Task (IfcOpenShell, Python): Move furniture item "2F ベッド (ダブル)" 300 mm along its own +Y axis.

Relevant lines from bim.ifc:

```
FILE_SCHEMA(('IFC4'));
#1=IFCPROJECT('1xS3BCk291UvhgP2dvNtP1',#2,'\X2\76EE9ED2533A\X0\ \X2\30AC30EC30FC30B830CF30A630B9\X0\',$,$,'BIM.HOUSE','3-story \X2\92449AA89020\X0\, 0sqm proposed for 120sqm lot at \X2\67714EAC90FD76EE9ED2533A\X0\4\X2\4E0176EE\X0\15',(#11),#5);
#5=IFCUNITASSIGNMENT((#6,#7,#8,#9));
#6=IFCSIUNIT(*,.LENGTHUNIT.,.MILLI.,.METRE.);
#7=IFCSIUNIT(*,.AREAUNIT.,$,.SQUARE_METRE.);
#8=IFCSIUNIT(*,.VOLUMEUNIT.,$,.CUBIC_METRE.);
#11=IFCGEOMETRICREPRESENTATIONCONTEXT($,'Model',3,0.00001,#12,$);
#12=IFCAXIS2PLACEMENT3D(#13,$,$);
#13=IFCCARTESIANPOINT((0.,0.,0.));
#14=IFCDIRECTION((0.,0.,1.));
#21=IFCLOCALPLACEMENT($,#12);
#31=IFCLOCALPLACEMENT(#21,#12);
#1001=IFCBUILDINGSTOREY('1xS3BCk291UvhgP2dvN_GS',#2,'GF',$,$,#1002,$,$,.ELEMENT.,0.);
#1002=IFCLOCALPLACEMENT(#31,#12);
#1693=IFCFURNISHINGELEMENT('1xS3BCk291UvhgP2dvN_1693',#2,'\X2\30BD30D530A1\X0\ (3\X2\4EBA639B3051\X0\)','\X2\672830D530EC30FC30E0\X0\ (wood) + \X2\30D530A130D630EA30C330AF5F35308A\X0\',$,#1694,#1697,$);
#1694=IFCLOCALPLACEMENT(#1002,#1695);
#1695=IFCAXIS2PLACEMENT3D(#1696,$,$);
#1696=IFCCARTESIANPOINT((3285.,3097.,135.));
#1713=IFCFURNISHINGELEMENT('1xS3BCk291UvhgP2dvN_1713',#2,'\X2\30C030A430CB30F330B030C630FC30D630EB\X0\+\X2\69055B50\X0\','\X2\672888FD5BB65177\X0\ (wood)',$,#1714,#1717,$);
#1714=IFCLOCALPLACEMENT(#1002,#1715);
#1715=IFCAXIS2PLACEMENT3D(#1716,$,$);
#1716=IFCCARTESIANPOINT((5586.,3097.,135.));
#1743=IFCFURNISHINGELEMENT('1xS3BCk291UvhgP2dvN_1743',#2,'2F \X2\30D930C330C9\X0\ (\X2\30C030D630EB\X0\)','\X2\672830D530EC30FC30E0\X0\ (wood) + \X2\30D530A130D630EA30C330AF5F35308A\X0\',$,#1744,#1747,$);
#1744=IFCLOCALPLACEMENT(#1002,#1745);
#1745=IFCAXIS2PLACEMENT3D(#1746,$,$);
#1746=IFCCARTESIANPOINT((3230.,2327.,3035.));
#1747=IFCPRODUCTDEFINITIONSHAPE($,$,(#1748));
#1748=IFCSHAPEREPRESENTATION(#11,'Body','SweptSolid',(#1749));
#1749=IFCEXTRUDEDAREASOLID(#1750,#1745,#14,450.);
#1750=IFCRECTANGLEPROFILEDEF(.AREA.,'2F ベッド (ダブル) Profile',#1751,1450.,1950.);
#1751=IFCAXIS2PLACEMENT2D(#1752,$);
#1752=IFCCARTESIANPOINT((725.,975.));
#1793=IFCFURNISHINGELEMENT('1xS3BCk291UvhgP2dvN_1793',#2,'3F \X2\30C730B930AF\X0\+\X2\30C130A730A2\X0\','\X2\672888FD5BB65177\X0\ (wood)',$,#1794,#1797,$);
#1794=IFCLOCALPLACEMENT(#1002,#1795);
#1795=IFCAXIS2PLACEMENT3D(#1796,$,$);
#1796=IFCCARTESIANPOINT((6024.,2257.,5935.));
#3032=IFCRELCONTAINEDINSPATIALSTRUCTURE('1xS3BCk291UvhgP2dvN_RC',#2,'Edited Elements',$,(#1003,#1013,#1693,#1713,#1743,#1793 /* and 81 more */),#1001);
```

```python
import ifcopenshell
import ifcopenshell.api.geometry
import ifcopenshell.util.placement
import ifcopenshell.util.unit

model = ifcopenshell.open("bim.ifc")
unit_scale = ifcopenshell.util.unit.calculate_unit_scale(model)

item = model.by_guid("1xS3BCk291UvhgP2dvN_1743")
matrix = ifcopenshell.util.placement.get_local_placement(item.ObjectPlacement)
matrix[:3, 3] += matrix[:3, 1] * 0.3 / unit_scale
ifcopenshell.api.geometry.edit_object_placement(model, product=item, matrix=matrix, is_si=False)

print(ifcopenshell.util.placement.get_local_placement(item.ObjectPlacement).round(3) + 0.0)

model.write("bim_rev.ifc")
```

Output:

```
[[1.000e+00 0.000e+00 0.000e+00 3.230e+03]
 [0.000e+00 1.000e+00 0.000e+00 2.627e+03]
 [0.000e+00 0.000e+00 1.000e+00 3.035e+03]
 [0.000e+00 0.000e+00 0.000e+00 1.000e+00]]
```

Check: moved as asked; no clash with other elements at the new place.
